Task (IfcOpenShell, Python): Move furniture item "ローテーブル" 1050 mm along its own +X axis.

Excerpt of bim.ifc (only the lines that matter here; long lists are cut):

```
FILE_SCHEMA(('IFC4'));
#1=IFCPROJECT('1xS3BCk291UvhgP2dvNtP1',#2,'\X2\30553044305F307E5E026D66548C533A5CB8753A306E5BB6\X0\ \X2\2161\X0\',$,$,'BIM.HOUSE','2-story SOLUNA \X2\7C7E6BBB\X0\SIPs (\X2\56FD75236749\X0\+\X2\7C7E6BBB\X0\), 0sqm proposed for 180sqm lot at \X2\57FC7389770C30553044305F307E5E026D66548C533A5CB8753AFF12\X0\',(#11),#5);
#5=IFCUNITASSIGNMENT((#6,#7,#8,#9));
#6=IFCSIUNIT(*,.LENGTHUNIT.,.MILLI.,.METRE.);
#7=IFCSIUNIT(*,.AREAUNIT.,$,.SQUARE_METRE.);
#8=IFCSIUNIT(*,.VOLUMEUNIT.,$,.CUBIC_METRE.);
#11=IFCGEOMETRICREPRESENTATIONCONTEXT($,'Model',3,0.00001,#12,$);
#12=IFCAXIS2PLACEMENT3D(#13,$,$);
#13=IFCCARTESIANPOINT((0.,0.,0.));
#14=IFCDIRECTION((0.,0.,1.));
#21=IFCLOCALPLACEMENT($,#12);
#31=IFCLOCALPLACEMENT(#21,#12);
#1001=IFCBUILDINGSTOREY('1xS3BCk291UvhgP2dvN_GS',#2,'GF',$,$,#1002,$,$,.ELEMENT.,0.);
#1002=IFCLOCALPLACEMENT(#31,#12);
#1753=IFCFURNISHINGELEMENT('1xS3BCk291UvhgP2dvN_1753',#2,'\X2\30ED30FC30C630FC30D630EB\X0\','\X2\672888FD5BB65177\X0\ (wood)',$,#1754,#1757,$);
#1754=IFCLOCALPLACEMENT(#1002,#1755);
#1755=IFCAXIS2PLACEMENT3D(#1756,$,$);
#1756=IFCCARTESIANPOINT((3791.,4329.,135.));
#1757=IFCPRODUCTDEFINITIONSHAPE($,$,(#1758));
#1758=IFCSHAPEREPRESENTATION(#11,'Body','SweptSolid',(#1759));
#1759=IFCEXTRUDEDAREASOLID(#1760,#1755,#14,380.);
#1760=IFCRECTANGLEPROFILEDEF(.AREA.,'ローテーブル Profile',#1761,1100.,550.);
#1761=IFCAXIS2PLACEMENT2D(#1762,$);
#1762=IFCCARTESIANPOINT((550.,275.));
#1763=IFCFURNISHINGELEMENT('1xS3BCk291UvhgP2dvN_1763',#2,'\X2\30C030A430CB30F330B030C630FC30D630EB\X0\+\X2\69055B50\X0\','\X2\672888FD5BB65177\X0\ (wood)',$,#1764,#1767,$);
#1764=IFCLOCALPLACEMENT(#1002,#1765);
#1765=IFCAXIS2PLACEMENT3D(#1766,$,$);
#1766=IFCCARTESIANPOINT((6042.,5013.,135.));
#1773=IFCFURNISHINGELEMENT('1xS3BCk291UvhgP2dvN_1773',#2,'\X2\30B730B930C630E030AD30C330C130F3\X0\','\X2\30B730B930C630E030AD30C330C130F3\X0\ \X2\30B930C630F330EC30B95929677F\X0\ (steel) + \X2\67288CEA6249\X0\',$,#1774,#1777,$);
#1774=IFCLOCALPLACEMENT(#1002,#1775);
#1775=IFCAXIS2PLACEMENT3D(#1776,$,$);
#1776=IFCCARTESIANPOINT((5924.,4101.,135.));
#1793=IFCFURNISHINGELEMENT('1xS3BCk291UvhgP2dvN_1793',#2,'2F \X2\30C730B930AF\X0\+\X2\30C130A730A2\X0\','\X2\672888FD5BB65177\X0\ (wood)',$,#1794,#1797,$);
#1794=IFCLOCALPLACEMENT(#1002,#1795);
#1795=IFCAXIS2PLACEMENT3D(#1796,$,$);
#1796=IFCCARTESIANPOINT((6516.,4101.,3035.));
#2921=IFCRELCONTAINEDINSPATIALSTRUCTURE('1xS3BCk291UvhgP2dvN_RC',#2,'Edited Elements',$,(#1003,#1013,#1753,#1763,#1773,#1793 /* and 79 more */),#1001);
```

```python
import ifcopenshell
import ifcopenshell.api.geometry
import ifcopenshell.util.placement

model = ifcopenshell.open("bim.ifc")

item = model.by_guid("1xS3BCk291UvhgP2dvN_1753")
matrix = ifcopenshell.util.placement.get_local_placement(item.ObjectPlacement)
matrix[:3, 3] += matrix[:3, 0] * 1050.0
ifcopenshell.api.geometry.edit_object_placement(model, product=item, matrix=matrix, is_si=False)

print(ifcopenshell.util.placement.get_local_placement(item.ObjectPlacement).round(3) + 0.0)

model.write("bim-out.ifc")
```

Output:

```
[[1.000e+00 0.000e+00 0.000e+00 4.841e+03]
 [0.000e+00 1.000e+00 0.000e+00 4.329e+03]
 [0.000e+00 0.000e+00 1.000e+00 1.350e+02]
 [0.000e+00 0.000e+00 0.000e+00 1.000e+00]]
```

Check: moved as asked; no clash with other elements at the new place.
